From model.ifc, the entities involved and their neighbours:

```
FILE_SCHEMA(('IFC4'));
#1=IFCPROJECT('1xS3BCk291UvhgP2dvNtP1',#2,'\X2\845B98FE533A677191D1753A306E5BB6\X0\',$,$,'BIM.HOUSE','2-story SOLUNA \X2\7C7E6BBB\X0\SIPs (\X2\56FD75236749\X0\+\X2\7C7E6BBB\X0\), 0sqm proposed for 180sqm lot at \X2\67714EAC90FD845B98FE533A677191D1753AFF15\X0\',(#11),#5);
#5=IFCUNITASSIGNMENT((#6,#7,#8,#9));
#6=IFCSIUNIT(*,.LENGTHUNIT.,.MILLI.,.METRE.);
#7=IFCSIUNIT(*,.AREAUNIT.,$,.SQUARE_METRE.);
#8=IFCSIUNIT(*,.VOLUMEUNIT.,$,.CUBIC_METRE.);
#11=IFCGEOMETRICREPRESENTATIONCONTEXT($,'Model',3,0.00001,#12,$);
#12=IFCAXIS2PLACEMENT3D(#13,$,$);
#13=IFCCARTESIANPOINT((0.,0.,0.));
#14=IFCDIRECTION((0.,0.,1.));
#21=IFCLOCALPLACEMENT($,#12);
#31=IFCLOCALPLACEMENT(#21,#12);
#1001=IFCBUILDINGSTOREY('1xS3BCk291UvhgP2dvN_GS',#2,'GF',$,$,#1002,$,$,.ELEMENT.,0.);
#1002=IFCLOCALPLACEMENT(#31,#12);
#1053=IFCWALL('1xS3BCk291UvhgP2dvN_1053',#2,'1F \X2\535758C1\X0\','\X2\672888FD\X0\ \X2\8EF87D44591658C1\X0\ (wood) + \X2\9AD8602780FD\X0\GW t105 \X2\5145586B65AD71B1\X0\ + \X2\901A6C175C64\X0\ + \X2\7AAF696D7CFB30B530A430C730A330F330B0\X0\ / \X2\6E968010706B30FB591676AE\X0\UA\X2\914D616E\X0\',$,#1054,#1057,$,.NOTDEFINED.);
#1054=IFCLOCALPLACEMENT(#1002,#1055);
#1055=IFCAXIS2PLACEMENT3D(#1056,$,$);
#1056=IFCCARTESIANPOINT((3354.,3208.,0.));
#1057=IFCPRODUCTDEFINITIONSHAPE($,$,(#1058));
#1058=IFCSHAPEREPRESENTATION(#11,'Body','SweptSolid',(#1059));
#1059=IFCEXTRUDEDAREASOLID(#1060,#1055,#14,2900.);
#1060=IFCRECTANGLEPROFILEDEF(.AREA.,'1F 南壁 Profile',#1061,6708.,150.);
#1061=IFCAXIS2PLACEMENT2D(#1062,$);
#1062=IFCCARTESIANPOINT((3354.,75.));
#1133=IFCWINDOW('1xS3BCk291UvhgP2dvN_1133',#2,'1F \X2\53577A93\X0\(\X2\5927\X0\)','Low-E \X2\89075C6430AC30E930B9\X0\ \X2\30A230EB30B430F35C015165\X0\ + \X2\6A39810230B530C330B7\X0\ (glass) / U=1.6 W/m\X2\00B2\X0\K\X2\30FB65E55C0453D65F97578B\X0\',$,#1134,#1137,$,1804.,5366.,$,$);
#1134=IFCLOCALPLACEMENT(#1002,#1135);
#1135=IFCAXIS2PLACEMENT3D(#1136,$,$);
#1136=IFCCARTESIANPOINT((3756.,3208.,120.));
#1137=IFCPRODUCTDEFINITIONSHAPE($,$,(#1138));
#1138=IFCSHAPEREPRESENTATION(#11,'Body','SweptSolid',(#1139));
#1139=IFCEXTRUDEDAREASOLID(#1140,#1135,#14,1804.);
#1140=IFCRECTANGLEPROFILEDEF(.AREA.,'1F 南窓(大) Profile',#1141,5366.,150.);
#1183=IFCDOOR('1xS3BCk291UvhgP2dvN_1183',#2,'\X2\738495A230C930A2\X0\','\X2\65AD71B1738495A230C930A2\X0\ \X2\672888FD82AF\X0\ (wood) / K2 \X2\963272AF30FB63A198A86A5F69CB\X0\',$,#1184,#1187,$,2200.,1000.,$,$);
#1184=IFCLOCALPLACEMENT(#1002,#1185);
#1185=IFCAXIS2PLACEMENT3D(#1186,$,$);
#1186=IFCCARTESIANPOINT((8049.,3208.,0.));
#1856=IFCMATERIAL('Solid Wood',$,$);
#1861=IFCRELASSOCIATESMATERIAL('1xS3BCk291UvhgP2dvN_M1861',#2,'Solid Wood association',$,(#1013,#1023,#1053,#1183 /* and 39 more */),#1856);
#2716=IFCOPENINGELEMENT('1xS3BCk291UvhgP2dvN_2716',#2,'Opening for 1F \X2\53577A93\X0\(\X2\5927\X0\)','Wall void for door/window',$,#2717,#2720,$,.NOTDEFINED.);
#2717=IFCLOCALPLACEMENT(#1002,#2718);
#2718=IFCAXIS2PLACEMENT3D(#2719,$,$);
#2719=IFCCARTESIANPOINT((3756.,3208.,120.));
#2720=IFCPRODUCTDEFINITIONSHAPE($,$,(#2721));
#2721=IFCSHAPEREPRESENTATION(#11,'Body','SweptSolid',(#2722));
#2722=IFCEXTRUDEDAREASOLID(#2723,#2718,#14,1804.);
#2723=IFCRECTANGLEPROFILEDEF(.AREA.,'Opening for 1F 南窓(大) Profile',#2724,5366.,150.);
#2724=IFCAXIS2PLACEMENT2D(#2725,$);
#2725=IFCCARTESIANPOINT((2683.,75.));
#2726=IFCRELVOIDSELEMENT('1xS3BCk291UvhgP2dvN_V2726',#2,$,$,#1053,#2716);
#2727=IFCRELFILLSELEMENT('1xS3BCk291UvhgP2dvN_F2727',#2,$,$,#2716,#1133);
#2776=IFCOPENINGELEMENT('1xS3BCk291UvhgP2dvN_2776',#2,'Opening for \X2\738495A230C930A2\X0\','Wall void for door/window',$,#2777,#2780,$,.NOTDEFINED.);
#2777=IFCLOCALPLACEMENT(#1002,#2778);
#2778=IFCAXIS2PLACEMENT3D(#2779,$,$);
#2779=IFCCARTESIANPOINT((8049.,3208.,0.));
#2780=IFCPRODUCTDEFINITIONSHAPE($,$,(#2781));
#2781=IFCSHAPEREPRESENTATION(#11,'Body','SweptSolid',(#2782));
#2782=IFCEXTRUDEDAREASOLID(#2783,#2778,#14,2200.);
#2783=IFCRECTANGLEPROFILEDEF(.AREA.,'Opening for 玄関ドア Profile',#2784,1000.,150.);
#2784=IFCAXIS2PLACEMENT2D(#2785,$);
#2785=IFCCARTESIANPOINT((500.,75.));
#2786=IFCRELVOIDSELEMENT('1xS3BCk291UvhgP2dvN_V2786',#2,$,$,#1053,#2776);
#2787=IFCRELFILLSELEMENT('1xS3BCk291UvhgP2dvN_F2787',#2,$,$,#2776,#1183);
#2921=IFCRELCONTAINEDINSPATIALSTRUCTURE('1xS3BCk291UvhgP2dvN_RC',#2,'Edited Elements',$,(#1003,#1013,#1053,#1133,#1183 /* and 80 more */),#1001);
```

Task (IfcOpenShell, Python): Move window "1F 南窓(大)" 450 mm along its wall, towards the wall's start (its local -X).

```python
import ifcopenshell
import ifcopenshell.api.geometry
import ifcopenshell.util.placement

model = ifcopenshell.open("model.ifc")

window = model.by_guid("1xS3BCk291UvhgP2dvN_1133")
opening = window.FillsVoids[0].RelatingOpeningElement
wall = opening.VoidsElements[0].RelatingBuildingElement

wall_matrix = ifcopenshell.util.placement.get_local_placement(wall.ObjectPlacement)
shift = wall_matrix[:3, 0] * -450.0
before = ifcopenshell.util.placement.get_local_placement(window.ObjectPlacement)[:3, 3].copy()

# The window is not placed relative to its opening, so move both.
for product in (opening, window):
    matrix = ifcopenshell.util.placement.get_local_placement(product.ObjectPlacement)
    matrix[:3, 3] += shift
    ifcopenshell.api.geometry.edit_object_placement(model, product=product, matrix=matrix, is_si=False)

after = ifcopenshell.util.placement.get_local_placement(window.ObjectPlacement)[:3, 3]
print("window moved by", (after - before).round(3) + 0.0)

model.write("model_edited.ifc")
```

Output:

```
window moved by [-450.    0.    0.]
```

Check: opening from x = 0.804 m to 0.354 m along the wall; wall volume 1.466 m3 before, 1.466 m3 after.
